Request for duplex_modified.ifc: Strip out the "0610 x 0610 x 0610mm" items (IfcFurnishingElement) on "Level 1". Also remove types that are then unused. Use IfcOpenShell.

First a look at what the model holds.

```python
import ifcopenshell
import ifcopenshell.util.element

model = ifcopenshell.open("duplex_modified.ifc")
print(model.schema)
storey = next(s for s in model.by_type("IfcBuildingStorey") if s.Name == "Level 1")
furniture = [e for e in ifcopenshell.util.element.get_decomposition(storey) if e.is_a("IfcFurnishingElement")]
seen = {}
for e in furniture:
    element_type = ifcopenshell.util.element.get_type(e)
    name = element_type.Name if element_type not in (None, e) else None
    seen[name] = seen.get(name, 0) + 1
for name, count in sorted(seen.items(), key=str):
    print(count, "x", name)
```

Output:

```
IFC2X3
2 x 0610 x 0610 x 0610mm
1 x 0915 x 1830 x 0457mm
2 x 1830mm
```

```python
import ifcopenshell
import ifcopenshell.api.root
import ifcopenshell.util.element

model = ifcopenshell.open("duplex_modified.ifc")

storey = next(s for s in model.by_type("IfcBuildingStorey") if s.Name == "Level 1")
furniture = [e for e in ifcopenshell.util.element.get_decomposition(storey) if e.is_a("IfcFurnishingElement")]
targets = [e for e in furniture if (t := ifcopenshell.util.element.get_type(e)) not in (None, e) and t.Name == "0610 x 0610 x 0610mm"]
types = {ifcopenshell.util.element.get_type(e) for e in targets} - {None, *targets}

for e in targets:
    ifcopenshell.api.root.remove_product(model, product=e)
print(len(targets), "removed")

unused = [t for t in types if not ifcopenshell.util.element.get_types(t)]
for t in unused:
    ifcopenshell.api.root.remove_product(model, product=t)
print(len(unused), "unused types removed")

model.write("duplex_modified_updated.ifc")
```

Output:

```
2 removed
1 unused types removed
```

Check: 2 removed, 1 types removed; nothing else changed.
